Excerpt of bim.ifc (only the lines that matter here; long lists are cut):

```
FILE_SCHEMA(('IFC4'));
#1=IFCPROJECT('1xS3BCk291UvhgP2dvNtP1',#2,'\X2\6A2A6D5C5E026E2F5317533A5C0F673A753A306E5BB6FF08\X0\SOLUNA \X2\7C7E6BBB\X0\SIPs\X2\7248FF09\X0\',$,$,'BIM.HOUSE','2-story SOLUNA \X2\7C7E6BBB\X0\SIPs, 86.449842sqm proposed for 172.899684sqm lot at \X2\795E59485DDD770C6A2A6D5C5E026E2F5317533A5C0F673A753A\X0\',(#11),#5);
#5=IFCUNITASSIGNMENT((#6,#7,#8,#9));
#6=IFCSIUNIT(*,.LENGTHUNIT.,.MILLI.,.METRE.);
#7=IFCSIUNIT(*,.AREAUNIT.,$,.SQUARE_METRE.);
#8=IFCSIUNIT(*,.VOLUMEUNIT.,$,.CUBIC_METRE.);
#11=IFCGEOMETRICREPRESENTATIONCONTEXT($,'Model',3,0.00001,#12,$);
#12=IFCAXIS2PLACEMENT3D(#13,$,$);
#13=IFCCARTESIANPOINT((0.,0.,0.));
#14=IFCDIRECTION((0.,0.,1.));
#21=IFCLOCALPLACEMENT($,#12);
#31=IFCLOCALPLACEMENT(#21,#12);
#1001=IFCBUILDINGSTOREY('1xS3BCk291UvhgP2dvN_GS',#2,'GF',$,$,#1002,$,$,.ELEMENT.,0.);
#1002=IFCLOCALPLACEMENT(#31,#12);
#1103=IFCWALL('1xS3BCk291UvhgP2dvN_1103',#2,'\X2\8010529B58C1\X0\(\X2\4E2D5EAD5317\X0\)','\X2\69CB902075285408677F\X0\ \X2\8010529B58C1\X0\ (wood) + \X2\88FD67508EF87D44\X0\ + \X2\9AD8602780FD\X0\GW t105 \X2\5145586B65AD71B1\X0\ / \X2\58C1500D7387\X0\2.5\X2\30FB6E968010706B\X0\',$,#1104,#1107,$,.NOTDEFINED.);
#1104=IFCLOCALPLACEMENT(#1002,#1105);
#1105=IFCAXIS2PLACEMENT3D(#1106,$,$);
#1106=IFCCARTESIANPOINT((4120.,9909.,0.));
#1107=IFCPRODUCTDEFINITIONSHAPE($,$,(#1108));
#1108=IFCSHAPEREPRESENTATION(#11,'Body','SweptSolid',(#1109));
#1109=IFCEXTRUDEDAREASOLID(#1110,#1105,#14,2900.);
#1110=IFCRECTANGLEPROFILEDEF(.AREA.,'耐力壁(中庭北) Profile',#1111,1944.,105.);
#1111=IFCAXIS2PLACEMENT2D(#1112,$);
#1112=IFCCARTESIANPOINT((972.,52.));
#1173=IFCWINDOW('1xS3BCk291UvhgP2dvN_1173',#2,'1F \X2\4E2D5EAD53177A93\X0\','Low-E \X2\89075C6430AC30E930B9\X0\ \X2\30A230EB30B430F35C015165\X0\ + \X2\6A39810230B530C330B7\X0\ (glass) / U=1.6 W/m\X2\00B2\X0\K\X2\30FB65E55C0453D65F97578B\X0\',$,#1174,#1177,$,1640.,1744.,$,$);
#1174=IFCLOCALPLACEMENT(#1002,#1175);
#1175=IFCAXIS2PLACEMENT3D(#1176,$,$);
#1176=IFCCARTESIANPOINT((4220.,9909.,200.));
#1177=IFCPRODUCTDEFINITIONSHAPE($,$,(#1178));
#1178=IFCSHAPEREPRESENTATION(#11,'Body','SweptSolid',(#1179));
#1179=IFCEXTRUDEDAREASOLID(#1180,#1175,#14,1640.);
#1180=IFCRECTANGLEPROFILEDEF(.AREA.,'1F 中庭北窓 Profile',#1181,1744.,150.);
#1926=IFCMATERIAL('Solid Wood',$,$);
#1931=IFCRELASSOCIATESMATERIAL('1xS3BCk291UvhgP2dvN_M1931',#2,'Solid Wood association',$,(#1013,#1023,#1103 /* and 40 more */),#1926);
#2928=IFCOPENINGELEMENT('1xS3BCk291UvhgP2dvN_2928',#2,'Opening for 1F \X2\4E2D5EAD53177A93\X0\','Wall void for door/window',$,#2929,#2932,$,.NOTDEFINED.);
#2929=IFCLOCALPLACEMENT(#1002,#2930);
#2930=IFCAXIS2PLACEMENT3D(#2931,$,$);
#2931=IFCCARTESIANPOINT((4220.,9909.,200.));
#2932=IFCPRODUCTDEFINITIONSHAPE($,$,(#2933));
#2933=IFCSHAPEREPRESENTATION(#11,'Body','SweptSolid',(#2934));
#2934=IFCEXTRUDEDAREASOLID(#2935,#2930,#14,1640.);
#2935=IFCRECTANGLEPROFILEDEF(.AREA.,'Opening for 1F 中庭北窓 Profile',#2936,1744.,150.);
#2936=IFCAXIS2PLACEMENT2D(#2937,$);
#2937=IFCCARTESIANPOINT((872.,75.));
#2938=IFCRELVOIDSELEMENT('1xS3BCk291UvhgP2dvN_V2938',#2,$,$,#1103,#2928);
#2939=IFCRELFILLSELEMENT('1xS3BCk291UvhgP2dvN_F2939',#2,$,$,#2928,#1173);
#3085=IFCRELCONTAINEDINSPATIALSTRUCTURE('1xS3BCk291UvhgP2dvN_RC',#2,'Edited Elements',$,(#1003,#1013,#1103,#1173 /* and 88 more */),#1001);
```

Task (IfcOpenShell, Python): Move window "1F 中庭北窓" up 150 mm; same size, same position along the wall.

```python
import numpy as np
import ifcopenshell
import ifcopenshell.api.geometry
import ifcopenshell.util.placement
import ifcopenshell.util.unit

model = ifcopenshell.open("bim.ifc")
unit_scale = ifcopenshell.util.unit.calculate_unit_scale(model)

window = model.by_guid("1xS3BCk291UvhgP2dvN_1173")
opening = window.FillsVoids[0].RelatingOpeningElement
dz = 0.15 / unit_scale

shift = np.array([0.0, 0.0, dz])
# The window is not placed relative to its opening, so move both.
for product in (opening, window):
    matrix = ifcopenshell.util.placement.get_local_placement(product.ObjectPlacement)
    matrix[:3, 3] += shift
    ifcopenshell.api.geometry.edit_object_placement(model, product=product, matrix=matrix, is_si=False)

print(f"moved by {dz * unit_scale:+.3f} m")

model.write("bim_v2.ifc")
```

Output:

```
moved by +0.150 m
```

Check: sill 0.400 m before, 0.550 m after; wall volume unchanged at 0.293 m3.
